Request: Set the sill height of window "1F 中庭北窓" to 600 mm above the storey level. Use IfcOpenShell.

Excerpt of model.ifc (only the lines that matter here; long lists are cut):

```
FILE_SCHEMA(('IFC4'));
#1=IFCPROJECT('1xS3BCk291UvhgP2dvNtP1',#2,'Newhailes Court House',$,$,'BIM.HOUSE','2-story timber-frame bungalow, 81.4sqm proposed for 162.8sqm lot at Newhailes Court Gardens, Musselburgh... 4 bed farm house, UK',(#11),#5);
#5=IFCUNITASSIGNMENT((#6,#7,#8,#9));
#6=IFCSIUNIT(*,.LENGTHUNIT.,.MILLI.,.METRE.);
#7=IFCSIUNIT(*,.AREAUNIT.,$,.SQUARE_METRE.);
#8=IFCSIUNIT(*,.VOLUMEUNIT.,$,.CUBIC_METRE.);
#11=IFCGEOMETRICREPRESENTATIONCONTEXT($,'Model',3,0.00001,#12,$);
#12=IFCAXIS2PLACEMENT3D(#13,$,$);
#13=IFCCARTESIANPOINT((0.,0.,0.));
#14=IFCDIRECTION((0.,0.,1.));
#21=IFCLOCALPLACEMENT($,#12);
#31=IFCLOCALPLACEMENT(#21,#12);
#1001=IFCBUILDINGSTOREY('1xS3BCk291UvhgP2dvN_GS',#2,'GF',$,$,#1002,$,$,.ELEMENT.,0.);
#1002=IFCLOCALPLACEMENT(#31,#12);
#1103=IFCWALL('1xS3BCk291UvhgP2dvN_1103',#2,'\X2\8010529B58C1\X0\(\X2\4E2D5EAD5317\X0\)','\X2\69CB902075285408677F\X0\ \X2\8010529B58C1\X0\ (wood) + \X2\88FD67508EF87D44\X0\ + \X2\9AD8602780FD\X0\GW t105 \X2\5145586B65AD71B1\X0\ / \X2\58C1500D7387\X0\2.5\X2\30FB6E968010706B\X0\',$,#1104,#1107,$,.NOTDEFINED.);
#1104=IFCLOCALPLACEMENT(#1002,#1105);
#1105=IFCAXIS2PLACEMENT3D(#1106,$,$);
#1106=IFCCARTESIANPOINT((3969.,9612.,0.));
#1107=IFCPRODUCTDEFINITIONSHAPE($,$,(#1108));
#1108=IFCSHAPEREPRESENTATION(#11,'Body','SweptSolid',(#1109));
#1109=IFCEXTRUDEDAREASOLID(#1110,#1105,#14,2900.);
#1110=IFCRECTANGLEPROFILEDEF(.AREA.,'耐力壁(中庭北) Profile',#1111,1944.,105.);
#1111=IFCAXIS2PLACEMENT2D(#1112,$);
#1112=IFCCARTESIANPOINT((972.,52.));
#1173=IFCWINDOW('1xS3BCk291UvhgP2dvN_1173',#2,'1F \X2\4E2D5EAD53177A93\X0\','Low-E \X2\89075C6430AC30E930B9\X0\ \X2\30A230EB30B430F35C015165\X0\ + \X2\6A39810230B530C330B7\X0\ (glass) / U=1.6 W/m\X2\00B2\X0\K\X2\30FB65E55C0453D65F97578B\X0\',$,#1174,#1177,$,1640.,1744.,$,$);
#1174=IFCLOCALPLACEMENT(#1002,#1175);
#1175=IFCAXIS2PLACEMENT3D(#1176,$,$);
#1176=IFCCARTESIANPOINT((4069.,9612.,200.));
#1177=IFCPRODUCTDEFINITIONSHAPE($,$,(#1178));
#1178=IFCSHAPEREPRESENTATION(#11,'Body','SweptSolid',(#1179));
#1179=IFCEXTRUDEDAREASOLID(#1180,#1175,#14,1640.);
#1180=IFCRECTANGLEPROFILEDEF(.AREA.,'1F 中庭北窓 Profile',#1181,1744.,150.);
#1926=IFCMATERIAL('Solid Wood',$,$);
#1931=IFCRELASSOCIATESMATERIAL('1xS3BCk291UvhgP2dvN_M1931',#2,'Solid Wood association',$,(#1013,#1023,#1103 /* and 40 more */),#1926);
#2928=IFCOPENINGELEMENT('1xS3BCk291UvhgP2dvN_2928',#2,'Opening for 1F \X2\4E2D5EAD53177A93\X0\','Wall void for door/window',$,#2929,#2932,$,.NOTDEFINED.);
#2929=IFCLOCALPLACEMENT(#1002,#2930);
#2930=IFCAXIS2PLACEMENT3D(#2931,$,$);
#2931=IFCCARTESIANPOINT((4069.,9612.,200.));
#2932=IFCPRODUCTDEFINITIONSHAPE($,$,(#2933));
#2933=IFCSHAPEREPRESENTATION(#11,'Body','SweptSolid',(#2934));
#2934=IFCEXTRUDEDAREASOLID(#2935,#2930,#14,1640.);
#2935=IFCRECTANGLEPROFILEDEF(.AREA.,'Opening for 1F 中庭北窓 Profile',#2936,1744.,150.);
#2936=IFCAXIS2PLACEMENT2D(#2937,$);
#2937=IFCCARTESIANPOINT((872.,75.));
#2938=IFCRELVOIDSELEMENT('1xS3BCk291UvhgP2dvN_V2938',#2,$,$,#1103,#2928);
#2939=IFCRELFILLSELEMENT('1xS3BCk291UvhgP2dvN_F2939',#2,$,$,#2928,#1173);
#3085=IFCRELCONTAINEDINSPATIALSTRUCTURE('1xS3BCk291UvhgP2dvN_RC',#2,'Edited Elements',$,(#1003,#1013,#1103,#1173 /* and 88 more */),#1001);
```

```python
import numpy as np
import ifcopenshell
import ifcopenshell.api.geometry
import ifcopenshell.geom
import ifcopenshell.util.element
import ifcopenshell.util.placement
import ifcopenshell.util.shape
import ifcopenshell.util.unit

model = ifcopenshell.open("model.ifc")
unit_scale = ifcopenshell.util.unit.calculate_unit_scale(model)

window = model.by_id(1173)
opening = window.FillsVoids[0].RelatingOpeningElement
storey = ifcopenshell.util.element.get_container(window, ifc_class="IfcBuildingStorey")
level = ifcopenshell.util.placement.get_local_placement(storey.ObjectPlacement)[2, 3]

# The opening's origin need not be at the sill, so measure its lowest point.
shape = ifcopenshell.geom.create_shape(ifcopenshell.geom.settings(), opening)
bottom = ifcopenshell.util.shape.get_shape_bottom_elevation(shape, shape.geometry) / unit_scale
dz = level + 600.0 - bottom

shift = np.array([0.0, 0.0, dz])
# The window is not placed relative to its opening, so move both.
for product in (opening, window):
    matrix = ifcopenshell.util.placement.get_local_placement(product.ObjectPlacement)
    matrix[:3, 3] += shift
    ifcopenshell.api.geometry.edit_object_placement(model, product=product, matrix=matrix, is_si=False)

print(f"moved by {dz * unit_scale:+.3f} m")

model.write("model_updated.ifc")
```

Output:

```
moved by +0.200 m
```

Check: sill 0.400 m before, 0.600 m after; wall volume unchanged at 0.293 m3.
